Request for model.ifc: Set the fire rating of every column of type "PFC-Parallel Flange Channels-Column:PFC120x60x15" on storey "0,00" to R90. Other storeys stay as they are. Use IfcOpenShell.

First a look at what the model holds.

```python
import ifcopenshell
import ifcopenshell.util.element

model = ifcopenshell.open("model.ifc")
print(model.schema)
storey = next(s for s in model.by_type("IfcBuildingStorey") if s.Name == "0,00")
columns = [e for e in ifcopenshell.util.element.get_decomposition(storey) if e.is_a("IfcColumn")]
seen = {}
for e in columns:
    element_type = ifcopenshell.util.element.get_type(e)
    key = (element_type.Name if element_type != e and element_type else None, ifcopenshell.util.element.get_pset(e, "Pset_ColumnCommon", "FireRating"))
    seen[key] = seen.get(key, 0) + 1
for (name, value), count in sorted(seen.items(), key=str):
    print(count, "x", name, "|", value)
```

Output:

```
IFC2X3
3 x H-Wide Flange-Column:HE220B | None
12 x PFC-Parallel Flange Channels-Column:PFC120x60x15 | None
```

```python
import ifcopenshell
import ifcopenshell.api.pset
import ifcopenshell.util.element

model = ifcopenshell.open("model.ifc")

storey = next(s for s in model.by_type("IfcBuildingStorey") if s.Name == "0,00")
columns = [e for e in ifcopenshell.util.element.get_decomposition(storey) if e.is_a("IfcColumn")]

count = 0
for e in columns:
    element_type = ifcopenshell.util.element.get_type(e)
    if element_type in (None, e) or element_type.Name != "PFC-Parallel Flange Channels-Column:PFC120x60x15":
        continue
    # add_pset returns the element's existing set when there is one.
    pset = ifcopenshell.api.pset.add_pset(model, product=e, name="Pset_ColumnCommon")
    ifcopenshell.api.pset.edit_pset(model, pset=pset, properties={"FireRating": "R90"})
    count += 1

print(count, "columns updated")

model.write("model_edited.ifc")
```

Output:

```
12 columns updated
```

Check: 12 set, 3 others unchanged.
